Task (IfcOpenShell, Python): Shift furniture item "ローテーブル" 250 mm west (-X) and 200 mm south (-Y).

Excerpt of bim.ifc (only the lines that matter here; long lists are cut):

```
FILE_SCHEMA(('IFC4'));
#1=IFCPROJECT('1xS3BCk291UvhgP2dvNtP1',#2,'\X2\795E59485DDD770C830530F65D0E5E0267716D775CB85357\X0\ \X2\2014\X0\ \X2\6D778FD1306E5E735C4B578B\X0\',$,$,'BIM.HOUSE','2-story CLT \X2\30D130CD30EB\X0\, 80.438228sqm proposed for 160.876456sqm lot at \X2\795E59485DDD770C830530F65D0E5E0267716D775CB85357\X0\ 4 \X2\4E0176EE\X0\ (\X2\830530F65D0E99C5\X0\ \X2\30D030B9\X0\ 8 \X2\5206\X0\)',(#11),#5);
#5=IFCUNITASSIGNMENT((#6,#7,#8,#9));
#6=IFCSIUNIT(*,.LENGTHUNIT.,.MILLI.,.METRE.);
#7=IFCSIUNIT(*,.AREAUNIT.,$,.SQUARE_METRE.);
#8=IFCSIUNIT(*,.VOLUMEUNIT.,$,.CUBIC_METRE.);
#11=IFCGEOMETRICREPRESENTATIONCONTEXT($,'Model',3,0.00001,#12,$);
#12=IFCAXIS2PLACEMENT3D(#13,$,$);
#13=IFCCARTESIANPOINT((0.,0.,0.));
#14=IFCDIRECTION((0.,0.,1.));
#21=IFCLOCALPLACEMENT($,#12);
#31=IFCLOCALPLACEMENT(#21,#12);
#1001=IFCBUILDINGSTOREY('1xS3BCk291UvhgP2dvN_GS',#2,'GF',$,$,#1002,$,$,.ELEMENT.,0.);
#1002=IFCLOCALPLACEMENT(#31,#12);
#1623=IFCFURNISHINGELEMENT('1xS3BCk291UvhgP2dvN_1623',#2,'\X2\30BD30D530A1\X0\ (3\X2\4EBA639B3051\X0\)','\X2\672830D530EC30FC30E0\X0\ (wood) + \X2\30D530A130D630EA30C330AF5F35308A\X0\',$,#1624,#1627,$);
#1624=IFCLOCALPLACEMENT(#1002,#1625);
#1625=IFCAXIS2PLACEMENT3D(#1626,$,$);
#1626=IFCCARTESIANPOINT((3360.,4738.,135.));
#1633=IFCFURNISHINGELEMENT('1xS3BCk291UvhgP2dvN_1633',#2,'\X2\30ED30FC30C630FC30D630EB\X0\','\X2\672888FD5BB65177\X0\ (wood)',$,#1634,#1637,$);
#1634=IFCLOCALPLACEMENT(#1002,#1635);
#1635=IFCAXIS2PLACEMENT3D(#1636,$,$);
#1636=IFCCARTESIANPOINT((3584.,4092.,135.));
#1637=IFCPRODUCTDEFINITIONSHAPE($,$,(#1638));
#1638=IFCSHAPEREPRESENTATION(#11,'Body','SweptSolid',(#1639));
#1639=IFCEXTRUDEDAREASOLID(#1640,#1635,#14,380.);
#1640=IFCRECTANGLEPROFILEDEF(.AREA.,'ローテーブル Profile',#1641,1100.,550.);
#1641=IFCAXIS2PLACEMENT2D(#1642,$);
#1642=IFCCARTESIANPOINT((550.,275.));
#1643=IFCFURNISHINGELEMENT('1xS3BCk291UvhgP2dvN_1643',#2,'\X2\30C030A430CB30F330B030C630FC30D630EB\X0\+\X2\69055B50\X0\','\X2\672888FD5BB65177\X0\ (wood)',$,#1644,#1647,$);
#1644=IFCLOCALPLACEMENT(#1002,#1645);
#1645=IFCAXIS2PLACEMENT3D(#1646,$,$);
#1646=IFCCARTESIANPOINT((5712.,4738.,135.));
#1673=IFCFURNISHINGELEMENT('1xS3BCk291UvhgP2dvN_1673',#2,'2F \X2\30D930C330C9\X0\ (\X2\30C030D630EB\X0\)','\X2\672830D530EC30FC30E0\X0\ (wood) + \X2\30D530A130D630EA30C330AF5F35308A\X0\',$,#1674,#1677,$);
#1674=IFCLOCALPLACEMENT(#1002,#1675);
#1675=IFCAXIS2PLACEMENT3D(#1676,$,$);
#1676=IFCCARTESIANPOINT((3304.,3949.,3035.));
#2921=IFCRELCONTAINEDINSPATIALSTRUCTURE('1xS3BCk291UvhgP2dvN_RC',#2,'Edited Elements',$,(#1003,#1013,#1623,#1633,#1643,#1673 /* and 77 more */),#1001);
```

```python
import ifcopenshell
import ifcopenshell.api.geometry
import ifcopenshell.util.placement
import ifcopenshell.util.unit

model = ifcopenshell.open("bim.ifc")
unit_scale = ifcopenshell.util.unit.calculate_unit_scale(model)

item = model.by_guid("1xS3BCk291UvhgP2dvN_1633")
matrix = ifcopenshell.util.placement.get_local_placement(item.ObjectPlacement)
matrix[0, 3] -= 0.25 / unit_scale
matrix[1, 3] -= 0.2 / unit_scale
ifcopenshell.api.geometry.edit_object_placement(model, product=item, matrix=matrix, is_si=False)

print(ifcopenshell.util.placement.get_local_placement(item.ObjectPlacement).round(3) + 0.0)

model.write("bim_updated.ifc")
```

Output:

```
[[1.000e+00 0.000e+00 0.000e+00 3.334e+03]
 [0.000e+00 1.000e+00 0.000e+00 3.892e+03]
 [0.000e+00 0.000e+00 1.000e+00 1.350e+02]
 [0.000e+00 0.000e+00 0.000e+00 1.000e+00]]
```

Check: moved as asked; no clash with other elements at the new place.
